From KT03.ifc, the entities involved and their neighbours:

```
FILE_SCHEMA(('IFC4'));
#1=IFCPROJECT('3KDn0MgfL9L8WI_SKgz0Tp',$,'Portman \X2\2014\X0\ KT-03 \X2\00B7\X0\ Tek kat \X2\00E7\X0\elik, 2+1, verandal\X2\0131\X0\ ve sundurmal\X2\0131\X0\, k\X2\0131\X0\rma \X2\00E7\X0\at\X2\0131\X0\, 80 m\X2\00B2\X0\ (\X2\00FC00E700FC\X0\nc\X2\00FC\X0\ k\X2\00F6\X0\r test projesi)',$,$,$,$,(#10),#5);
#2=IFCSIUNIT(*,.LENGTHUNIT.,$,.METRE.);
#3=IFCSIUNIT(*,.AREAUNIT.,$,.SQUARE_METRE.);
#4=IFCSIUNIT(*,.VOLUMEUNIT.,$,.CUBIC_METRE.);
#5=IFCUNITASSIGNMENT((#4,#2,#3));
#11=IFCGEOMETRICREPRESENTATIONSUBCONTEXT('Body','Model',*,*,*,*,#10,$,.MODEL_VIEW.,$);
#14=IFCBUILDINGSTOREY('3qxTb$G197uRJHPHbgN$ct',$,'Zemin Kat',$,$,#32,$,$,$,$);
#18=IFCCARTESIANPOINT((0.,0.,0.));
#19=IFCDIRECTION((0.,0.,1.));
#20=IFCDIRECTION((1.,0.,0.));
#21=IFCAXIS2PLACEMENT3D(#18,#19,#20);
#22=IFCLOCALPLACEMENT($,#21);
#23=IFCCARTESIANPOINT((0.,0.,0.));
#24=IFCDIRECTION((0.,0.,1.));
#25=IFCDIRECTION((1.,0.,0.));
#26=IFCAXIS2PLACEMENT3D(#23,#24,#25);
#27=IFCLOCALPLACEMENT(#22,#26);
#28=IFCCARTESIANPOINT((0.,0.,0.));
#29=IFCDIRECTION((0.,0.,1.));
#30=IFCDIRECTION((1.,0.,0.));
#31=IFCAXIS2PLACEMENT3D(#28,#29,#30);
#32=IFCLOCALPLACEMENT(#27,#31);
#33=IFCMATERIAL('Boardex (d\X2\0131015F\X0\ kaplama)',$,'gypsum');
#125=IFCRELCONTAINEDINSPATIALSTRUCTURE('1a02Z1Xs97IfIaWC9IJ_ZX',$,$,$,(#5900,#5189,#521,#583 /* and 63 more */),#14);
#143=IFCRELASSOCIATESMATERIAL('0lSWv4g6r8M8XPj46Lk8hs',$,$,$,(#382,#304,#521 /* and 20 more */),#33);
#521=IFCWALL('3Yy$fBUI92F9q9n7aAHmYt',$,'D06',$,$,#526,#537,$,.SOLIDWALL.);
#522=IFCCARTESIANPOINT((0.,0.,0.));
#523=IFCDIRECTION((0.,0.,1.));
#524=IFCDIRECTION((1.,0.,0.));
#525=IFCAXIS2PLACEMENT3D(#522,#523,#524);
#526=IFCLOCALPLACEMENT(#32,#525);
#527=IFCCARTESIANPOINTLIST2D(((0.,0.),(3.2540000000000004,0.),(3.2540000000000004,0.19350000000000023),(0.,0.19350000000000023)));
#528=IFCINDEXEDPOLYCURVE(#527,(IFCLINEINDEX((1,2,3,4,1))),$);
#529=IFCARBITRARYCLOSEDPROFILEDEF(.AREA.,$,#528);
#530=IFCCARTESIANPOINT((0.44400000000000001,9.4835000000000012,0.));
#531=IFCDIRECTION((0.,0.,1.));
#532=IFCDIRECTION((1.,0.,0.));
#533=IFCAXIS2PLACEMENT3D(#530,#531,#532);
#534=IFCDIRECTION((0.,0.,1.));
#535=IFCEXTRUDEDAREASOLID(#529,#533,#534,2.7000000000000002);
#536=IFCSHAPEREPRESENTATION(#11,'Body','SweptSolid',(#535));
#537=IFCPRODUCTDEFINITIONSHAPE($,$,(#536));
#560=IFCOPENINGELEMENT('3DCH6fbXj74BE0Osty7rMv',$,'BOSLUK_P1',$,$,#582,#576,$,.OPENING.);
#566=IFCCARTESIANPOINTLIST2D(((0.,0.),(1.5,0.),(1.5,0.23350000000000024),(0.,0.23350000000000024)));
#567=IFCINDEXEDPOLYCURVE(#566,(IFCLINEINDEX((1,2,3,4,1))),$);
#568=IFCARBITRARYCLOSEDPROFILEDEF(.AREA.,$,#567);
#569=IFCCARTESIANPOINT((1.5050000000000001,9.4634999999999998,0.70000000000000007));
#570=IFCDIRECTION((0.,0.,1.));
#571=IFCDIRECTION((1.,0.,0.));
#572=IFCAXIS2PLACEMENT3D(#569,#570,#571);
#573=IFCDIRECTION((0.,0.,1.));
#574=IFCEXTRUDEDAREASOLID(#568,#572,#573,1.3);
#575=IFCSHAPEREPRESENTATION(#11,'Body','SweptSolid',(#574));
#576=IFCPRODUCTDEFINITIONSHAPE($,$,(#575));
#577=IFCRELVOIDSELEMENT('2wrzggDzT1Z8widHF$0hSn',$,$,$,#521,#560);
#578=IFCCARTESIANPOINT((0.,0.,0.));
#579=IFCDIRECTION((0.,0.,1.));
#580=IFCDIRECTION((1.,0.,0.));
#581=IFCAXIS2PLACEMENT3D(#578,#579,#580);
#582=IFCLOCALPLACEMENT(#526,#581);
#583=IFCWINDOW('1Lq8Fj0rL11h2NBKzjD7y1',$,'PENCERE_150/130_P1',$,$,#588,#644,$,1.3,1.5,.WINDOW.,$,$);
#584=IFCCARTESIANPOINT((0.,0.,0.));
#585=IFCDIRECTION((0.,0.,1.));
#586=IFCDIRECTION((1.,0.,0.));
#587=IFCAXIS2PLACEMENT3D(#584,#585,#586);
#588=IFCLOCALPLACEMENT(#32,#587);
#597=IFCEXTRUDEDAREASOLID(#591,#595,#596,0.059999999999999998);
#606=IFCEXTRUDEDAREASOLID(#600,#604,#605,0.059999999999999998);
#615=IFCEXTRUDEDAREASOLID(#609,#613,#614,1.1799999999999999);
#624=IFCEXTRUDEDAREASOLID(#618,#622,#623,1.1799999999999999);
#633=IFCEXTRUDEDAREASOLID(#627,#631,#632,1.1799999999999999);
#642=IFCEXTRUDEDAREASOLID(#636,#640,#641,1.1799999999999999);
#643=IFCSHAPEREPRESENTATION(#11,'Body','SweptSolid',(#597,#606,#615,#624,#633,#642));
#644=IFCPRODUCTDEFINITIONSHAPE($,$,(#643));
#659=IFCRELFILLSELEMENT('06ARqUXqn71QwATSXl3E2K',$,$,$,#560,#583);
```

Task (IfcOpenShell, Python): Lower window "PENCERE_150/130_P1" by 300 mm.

```python
import numpy as np
import ifcopenshell
import ifcopenshell.api.geometry
import ifcopenshell.util.placement
import ifcopenshell.util.unit

model = ifcopenshell.open("KT03.ifc")
unit_scale = ifcopenshell.util.unit.calculate_unit_scale(model)

window = model.by_guid("1Lq8Fj0rL11h2NBKzjD7y1")
opening = window.FillsVoids[0].RelatingOpeningElement
dz = -0.3 / unit_scale

shift = np.array([0.0, 0.0, dz])
# The window is not placed relative to its opening, so move both.
for product in (opening, window):
    matrix = ifcopenshell.util.placement.get_local_placement(product.ObjectPlacement)
    matrix[:3, 3] += shift
    ifcopenshell.api.geometry.edit_object_placement(model, product=product, matrix=matrix, is_si=False)

print(f"moved by {dz * unit_scale:+.3f} m")

model.write("KT03_edited.ifc")
```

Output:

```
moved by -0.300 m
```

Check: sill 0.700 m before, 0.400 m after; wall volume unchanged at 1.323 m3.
